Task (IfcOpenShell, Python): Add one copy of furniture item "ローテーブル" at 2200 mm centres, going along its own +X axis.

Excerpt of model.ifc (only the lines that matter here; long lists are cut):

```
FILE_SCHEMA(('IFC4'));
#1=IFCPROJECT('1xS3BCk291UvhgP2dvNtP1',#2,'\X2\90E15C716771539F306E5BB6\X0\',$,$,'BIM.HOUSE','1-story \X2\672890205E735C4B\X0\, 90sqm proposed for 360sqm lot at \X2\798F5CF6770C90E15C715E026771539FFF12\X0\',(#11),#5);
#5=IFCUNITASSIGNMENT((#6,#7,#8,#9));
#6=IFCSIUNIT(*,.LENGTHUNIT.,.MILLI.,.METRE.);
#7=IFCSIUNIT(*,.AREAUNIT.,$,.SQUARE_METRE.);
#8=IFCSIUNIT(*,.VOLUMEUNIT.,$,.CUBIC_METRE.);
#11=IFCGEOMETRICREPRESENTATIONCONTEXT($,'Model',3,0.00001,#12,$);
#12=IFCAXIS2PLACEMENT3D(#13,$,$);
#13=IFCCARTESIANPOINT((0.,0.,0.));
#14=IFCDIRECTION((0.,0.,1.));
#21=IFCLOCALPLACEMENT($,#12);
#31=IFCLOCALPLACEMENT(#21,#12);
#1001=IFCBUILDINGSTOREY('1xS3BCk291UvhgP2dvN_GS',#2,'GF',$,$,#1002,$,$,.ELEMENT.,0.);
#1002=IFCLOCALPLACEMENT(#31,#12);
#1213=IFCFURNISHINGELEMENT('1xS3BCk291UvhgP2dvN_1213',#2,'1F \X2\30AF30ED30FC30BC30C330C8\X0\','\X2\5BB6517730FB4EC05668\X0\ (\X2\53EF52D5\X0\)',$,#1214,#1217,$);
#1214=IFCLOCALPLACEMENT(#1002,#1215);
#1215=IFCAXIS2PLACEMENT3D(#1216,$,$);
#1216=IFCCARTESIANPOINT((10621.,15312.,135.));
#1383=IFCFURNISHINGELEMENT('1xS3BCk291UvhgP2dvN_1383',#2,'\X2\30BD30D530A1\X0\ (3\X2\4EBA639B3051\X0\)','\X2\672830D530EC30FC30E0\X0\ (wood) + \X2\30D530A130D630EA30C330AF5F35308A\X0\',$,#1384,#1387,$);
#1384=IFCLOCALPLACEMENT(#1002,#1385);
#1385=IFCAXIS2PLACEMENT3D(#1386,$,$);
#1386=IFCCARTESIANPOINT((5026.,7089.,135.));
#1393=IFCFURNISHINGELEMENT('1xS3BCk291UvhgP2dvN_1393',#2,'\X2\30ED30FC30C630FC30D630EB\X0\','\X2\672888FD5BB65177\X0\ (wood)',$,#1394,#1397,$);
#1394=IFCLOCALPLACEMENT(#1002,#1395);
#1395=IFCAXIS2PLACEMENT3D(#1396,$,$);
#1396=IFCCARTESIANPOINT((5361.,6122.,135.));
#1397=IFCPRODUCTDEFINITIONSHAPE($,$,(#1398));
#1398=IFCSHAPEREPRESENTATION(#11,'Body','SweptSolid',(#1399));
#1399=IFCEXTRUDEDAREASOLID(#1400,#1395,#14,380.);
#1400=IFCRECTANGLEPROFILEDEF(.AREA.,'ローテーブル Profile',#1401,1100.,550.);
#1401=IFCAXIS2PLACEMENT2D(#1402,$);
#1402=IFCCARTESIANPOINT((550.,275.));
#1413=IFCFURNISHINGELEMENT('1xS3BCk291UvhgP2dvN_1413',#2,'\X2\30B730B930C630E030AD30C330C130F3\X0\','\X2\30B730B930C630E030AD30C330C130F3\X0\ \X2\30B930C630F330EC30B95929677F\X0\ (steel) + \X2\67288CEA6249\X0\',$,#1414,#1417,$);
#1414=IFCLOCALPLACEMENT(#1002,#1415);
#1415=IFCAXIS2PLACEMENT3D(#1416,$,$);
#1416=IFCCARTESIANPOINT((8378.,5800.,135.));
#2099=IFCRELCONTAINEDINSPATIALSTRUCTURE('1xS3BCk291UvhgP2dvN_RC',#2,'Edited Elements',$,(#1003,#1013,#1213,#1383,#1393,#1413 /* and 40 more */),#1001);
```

```python
import ifcopenshell
import ifcopenshell.api.geometry
import ifcopenshell.api.root
import ifcopenshell.util.element
import ifcopenshell.util.placement
import ifcopenshell.util.unit

model = ifcopenshell.open("model.ifc")
unit_scale = ifcopenshell.util.unit.calculate_unit_scale(model)


def reuse_history(source, copy):
    """copy_class also copies each property set's owner history, people and application; keep the originals."""
    for rel in copy.IsDefinedBy:
        if rel.is_a("IfcRelDefinesByProperties") and (history := rel.RelatingPropertyDefinition.OwnerHistory):
            rel.RelatingPropertyDefinition.OwnerHistory = source.OwnerHistory
            ifcopenshell.util.element.remove_deep2(model, history)


source = model.by_guid("1xS3BCk291UvhgP2dvN_1393")
base = ifcopenshell.util.placement.get_local_placement(source.ObjectPlacement)
step = base[:3, 0] * 2.2 / unit_scale

for i in range(1, 2):
    copy = ifcopenshell.api.root.copy_class(model, product=source)
    copy.Representation = ifcopenshell.util.element.copy_deep(
        model, source.Representation, exclude=["IfcGeometricRepresentationContext", "IfcRepresentationMap"]
    )
    reuse_history(source, copy)
    matrix = base.copy()
    matrix[:3, 3] += i * step
    print("added at", matrix[:3, 3].round(3) + 0.0)
    ifcopenshell.api.geometry.edit_object_placement(model, product=copy, matrix=matrix, is_si=False)

model.write("model_edited.ifc")
```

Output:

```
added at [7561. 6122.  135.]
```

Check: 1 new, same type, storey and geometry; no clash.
